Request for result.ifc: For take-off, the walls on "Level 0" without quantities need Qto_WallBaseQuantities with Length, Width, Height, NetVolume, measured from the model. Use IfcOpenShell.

First a look at what the model holds.

```python
import ifcopenshell
import ifcopenshell.util.element
import ifcopenshell.util.unit

model = ifcopenshell.open("result.ifc")
print(model.schema)
for unit_type in ("LENGTHUNIT", "AREAUNIT", "VOLUMEUNIT"):
    print(unit_type, ifcopenshell.util.unit.calculate_unit_scale(model, unit_type))
storey = next(s for s in model.by_type("IfcBuildingStorey") if s.Name == "Level 0")
walls = [e for e in ifcopenshell.util.element.get_decomposition(storey) if e.is_a("IfcWall")]
for e in sorted(walls, key=lambda e: e.id()):
    print(e.id(), e.is_a(), e.Name, list(ifcopenshell.util.element.get_psets(e, qtos_only=True)), sep=" | ")
```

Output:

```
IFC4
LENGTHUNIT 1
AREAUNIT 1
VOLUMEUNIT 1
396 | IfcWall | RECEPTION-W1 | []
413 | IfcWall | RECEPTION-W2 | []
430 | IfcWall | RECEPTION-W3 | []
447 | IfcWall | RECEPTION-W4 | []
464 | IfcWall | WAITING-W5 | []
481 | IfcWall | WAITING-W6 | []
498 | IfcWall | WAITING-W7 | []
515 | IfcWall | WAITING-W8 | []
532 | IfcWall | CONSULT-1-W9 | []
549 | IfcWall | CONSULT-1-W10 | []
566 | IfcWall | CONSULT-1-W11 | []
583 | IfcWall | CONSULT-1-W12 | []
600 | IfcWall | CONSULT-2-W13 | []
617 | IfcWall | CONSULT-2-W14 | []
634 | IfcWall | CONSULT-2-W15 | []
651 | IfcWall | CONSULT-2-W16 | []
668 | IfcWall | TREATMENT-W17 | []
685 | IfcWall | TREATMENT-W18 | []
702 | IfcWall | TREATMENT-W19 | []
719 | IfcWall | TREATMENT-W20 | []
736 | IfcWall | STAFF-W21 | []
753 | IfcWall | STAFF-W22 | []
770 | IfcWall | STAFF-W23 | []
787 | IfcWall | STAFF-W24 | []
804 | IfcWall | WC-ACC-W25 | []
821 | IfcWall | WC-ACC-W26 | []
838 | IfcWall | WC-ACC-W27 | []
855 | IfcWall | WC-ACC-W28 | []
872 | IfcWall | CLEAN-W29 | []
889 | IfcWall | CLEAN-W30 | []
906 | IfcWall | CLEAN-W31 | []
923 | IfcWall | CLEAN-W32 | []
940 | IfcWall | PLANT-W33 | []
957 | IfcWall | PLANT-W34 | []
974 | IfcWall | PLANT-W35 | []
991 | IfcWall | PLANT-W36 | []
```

```python
import ifcopenshell
import ifcopenshell.api.pset
import ifcopenshell.geom
import ifcopenshell.util.element
import ifcopenshell.util.shape
import ifcopenshell.util.unit

model = ifcopenshell.open("result.ifc")
unit_scale = ifcopenshell.util.unit.calculate_unit_scale(model)
volume_scale = ifcopenshell.util.unit.calculate_unit_scale(model, "VOLUMEUNIT")
settings = ifcopenshell.geom.settings()

storey = next(s for s in model.by_type("IfcBuildingStorey") if s.Name == "Level 0")
walls = [e for e in ifcopenshell.util.element.get_decomposition(storey) if e.is_a("IfcWall")]

for e in sorted(walls, key=lambda e: e.id()):
    if ifcopenshell.util.element.get_psets(e, qtos_only=True, should_inherit=False):
        continue
    # Geometry comes back in metres, in the element's own axes.
    shape = ifcopenshell.geom.create_shape(settings, e)
    values = {
        "Length": ifcopenshell.util.shape.get_x(shape.geometry) / unit_scale,
        "Width": ifcopenshell.util.shape.get_y(shape.geometry) / unit_scale,
        "Height": ifcopenshell.util.shape.get_z(shape.geometry) / unit_scale,
        "NetVolume": ifcopenshell.util.shape.get_volume(shape.geometry) / volume_scale,
    }
    qto = ifcopenshell.api.pset.add_qto(model, product=e, name="Qto_WallBaseQuantities")
    ifcopenshell.api.pset.edit_qto(model, qto=qto, properties=values)
    print(e.id(), {k: round(v, 3) for k, v in values.items()})

model.write("result_edited.ifc")
```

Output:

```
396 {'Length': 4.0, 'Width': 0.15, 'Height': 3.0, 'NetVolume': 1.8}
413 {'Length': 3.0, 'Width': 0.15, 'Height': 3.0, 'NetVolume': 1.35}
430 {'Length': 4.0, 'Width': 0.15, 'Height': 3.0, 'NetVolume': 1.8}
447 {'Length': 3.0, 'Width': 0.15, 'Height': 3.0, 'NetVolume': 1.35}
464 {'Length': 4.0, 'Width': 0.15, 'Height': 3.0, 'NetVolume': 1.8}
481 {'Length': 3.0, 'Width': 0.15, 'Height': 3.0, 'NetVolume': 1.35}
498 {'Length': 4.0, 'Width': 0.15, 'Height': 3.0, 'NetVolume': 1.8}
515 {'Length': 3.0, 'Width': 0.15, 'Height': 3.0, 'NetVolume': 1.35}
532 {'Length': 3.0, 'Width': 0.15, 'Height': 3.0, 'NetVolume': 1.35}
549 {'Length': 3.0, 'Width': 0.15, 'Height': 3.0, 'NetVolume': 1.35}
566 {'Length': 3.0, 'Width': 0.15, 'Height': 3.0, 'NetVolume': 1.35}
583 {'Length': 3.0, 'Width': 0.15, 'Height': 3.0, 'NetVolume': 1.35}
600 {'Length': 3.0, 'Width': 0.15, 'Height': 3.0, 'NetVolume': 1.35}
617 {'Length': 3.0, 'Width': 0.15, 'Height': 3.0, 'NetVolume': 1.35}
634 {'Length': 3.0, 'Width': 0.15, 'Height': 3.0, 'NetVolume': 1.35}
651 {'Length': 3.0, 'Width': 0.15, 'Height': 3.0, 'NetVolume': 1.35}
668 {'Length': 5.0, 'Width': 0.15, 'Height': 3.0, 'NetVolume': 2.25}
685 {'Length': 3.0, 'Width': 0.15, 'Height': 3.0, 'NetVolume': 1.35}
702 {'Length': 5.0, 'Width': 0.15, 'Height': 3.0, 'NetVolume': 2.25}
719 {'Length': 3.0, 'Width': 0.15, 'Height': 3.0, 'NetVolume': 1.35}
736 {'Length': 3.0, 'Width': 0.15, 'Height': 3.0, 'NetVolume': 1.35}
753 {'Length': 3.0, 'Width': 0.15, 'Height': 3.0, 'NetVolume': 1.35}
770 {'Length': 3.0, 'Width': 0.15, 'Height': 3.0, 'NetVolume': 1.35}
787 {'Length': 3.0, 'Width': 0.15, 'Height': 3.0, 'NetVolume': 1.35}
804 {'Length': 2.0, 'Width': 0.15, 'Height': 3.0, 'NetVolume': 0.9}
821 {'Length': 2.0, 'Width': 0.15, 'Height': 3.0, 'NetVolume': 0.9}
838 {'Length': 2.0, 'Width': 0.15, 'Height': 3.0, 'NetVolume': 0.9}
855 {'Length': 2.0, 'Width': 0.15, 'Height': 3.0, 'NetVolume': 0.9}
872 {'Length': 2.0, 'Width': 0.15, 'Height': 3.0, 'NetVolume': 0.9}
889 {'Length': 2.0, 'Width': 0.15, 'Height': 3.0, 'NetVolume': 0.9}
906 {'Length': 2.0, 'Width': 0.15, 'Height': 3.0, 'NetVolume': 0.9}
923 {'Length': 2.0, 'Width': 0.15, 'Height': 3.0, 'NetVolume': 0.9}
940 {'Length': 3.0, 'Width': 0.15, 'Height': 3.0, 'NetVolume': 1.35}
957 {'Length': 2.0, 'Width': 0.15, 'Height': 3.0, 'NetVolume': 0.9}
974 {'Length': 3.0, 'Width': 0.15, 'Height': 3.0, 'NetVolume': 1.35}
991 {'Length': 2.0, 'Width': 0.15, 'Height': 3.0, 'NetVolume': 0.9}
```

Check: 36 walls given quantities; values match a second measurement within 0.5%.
